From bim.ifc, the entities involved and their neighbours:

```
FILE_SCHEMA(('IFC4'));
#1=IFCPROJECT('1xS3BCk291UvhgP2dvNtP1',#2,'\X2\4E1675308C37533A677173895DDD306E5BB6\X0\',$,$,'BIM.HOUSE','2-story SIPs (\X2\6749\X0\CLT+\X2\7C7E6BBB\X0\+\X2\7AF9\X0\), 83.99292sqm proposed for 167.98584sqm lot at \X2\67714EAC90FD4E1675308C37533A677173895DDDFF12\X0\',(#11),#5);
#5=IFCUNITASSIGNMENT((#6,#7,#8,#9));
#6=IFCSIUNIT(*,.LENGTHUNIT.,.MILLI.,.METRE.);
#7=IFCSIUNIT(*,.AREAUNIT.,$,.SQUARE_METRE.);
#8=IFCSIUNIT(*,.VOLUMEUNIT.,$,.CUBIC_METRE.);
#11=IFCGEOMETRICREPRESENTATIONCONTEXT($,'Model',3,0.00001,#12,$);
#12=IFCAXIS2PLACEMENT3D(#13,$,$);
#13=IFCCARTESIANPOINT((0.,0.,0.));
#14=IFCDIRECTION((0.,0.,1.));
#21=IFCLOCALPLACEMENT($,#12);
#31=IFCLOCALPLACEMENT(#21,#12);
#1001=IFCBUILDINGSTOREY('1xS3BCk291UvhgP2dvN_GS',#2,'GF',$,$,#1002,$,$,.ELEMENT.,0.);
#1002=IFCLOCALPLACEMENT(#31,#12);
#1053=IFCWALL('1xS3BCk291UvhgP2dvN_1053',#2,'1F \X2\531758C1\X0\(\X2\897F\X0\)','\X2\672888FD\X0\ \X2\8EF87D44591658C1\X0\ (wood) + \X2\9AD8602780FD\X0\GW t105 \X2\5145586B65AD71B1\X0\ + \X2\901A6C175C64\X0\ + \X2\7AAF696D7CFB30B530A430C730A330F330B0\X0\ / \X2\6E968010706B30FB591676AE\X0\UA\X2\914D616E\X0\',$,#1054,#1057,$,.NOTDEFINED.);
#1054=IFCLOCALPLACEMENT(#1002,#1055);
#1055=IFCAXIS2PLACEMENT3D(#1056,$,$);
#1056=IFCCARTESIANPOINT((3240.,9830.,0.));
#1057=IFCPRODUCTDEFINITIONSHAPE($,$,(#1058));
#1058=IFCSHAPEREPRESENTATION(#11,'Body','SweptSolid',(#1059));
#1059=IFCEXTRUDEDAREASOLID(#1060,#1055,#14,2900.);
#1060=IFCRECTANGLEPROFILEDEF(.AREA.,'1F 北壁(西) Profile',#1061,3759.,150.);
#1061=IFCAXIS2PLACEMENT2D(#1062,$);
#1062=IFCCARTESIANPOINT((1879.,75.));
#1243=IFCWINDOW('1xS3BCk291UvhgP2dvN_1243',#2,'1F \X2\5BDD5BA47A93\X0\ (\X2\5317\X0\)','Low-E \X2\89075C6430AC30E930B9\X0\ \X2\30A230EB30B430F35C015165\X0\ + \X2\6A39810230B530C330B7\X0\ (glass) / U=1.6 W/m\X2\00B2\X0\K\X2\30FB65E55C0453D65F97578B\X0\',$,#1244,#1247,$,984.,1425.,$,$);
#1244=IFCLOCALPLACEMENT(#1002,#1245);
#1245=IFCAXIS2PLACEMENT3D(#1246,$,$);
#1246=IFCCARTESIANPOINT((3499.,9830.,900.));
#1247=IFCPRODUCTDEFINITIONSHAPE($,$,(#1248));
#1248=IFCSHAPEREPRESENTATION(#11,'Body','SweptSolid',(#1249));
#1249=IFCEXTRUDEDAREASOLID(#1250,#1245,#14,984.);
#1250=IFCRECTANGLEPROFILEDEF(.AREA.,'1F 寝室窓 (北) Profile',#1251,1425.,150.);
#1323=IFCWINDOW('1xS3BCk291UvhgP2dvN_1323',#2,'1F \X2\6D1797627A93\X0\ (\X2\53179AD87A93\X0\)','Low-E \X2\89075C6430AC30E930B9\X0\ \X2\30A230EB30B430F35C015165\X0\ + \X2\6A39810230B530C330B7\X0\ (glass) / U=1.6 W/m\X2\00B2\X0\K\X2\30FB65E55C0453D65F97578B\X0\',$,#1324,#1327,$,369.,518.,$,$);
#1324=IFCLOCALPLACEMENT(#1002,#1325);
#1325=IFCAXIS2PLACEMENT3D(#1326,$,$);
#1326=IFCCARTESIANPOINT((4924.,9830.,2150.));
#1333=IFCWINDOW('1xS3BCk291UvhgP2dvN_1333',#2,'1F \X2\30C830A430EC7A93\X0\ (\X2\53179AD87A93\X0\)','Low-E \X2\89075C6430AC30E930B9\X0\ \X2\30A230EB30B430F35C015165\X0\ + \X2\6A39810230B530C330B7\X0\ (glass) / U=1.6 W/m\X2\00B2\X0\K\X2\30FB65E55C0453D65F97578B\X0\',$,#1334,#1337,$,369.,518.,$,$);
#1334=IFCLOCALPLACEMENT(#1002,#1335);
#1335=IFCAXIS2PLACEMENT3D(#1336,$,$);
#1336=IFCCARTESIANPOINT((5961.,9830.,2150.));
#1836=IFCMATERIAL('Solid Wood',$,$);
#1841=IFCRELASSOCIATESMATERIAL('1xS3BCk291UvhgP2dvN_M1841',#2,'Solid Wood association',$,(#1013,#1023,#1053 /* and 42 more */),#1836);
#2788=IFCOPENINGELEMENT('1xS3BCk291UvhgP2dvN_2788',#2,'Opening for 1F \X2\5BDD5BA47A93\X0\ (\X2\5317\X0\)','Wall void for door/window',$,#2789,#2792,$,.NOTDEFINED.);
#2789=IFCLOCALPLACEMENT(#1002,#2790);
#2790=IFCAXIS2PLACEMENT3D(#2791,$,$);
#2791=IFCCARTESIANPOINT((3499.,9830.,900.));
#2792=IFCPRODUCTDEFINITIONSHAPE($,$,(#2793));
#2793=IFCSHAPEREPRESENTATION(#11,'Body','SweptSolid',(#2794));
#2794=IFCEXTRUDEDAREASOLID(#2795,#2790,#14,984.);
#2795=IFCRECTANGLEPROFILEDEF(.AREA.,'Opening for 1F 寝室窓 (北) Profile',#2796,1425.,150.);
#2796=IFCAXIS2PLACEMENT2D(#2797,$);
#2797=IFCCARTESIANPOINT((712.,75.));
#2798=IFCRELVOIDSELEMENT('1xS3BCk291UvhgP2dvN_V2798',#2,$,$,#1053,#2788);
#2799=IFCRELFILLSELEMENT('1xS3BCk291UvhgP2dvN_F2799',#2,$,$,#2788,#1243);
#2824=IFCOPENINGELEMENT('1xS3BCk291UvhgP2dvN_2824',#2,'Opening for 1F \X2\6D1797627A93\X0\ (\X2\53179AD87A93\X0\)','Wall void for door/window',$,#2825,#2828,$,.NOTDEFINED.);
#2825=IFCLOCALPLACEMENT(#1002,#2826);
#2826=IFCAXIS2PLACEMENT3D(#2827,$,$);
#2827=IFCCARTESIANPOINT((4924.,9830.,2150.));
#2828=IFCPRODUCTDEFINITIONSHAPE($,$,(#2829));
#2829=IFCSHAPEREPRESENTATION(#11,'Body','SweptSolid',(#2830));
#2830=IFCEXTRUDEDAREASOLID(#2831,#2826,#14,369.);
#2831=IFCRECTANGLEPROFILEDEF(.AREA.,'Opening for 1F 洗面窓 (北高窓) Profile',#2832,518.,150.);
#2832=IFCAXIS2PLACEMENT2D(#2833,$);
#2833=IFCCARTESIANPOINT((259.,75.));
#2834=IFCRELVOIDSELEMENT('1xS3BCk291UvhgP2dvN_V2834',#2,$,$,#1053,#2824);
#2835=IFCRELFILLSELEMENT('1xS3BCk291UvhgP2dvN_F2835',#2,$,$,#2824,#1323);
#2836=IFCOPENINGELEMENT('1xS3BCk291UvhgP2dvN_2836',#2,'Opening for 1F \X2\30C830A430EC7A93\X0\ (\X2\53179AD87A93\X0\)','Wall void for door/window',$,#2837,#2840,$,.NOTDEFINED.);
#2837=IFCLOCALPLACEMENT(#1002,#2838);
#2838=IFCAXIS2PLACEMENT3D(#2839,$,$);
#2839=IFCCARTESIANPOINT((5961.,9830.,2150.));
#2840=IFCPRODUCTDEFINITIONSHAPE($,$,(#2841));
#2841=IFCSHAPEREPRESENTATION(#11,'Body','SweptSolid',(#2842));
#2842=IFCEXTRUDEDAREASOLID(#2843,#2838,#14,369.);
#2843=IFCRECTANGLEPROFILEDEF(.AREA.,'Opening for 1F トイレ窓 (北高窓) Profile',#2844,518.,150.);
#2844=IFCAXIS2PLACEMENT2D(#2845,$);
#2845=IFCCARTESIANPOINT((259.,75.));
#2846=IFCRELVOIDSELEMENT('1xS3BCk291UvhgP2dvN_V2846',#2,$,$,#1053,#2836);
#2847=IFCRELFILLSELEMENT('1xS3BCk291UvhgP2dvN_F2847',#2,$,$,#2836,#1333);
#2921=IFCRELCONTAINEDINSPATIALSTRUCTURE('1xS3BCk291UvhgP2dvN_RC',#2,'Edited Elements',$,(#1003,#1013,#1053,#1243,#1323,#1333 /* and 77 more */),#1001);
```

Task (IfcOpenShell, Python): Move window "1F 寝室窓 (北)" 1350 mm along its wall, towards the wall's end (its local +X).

```python
import ifcopenshell
import ifcopenshell.api.geometry
import ifcopenshell.util.placement
import ifcopenshell.util.unit

model = ifcopenshell.open("bim.ifc")
unit_scale = ifcopenshell.util.unit.calculate_unit_scale(model)

window = model.by_guid("1xS3BCk291UvhgP2dvN_1243")
opening = window.FillsVoids[0].RelatingOpeningElement
wall = opening.VoidsElements[0].RelatingBuildingElement

wall_matrix = ifcopenshell.util.placement.get_local_placement(wall.ObjectPlacement)
shift = wall_matrix[:3, 0] * 1.35 / unit_scale
before = ifcopenshell.util.placement.get_local_placement(window.ObjectPlacement)[:3, 3].copy()

# The window is not placed relative to its opening, so move both.
for product in (opening, window):
    matrix = ifcopenshell.util.placement.get_local_placement(product.ObjectPlacement)
    matrix[:3, 3] += shift
    ifcopenshell.api.geometry.edit_object_placement(model, product=product, matrix=matrix, is_si=False)

after = ifcopenshell.util.placement.get_local_placement(window.ObjectPlacement)[:3, 3]
print("window moved by", (after - before).round(3) + 0.0)

model.write("bim-out.ifc")
```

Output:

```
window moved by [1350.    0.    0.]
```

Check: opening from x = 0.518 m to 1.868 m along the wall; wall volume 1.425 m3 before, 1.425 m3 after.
